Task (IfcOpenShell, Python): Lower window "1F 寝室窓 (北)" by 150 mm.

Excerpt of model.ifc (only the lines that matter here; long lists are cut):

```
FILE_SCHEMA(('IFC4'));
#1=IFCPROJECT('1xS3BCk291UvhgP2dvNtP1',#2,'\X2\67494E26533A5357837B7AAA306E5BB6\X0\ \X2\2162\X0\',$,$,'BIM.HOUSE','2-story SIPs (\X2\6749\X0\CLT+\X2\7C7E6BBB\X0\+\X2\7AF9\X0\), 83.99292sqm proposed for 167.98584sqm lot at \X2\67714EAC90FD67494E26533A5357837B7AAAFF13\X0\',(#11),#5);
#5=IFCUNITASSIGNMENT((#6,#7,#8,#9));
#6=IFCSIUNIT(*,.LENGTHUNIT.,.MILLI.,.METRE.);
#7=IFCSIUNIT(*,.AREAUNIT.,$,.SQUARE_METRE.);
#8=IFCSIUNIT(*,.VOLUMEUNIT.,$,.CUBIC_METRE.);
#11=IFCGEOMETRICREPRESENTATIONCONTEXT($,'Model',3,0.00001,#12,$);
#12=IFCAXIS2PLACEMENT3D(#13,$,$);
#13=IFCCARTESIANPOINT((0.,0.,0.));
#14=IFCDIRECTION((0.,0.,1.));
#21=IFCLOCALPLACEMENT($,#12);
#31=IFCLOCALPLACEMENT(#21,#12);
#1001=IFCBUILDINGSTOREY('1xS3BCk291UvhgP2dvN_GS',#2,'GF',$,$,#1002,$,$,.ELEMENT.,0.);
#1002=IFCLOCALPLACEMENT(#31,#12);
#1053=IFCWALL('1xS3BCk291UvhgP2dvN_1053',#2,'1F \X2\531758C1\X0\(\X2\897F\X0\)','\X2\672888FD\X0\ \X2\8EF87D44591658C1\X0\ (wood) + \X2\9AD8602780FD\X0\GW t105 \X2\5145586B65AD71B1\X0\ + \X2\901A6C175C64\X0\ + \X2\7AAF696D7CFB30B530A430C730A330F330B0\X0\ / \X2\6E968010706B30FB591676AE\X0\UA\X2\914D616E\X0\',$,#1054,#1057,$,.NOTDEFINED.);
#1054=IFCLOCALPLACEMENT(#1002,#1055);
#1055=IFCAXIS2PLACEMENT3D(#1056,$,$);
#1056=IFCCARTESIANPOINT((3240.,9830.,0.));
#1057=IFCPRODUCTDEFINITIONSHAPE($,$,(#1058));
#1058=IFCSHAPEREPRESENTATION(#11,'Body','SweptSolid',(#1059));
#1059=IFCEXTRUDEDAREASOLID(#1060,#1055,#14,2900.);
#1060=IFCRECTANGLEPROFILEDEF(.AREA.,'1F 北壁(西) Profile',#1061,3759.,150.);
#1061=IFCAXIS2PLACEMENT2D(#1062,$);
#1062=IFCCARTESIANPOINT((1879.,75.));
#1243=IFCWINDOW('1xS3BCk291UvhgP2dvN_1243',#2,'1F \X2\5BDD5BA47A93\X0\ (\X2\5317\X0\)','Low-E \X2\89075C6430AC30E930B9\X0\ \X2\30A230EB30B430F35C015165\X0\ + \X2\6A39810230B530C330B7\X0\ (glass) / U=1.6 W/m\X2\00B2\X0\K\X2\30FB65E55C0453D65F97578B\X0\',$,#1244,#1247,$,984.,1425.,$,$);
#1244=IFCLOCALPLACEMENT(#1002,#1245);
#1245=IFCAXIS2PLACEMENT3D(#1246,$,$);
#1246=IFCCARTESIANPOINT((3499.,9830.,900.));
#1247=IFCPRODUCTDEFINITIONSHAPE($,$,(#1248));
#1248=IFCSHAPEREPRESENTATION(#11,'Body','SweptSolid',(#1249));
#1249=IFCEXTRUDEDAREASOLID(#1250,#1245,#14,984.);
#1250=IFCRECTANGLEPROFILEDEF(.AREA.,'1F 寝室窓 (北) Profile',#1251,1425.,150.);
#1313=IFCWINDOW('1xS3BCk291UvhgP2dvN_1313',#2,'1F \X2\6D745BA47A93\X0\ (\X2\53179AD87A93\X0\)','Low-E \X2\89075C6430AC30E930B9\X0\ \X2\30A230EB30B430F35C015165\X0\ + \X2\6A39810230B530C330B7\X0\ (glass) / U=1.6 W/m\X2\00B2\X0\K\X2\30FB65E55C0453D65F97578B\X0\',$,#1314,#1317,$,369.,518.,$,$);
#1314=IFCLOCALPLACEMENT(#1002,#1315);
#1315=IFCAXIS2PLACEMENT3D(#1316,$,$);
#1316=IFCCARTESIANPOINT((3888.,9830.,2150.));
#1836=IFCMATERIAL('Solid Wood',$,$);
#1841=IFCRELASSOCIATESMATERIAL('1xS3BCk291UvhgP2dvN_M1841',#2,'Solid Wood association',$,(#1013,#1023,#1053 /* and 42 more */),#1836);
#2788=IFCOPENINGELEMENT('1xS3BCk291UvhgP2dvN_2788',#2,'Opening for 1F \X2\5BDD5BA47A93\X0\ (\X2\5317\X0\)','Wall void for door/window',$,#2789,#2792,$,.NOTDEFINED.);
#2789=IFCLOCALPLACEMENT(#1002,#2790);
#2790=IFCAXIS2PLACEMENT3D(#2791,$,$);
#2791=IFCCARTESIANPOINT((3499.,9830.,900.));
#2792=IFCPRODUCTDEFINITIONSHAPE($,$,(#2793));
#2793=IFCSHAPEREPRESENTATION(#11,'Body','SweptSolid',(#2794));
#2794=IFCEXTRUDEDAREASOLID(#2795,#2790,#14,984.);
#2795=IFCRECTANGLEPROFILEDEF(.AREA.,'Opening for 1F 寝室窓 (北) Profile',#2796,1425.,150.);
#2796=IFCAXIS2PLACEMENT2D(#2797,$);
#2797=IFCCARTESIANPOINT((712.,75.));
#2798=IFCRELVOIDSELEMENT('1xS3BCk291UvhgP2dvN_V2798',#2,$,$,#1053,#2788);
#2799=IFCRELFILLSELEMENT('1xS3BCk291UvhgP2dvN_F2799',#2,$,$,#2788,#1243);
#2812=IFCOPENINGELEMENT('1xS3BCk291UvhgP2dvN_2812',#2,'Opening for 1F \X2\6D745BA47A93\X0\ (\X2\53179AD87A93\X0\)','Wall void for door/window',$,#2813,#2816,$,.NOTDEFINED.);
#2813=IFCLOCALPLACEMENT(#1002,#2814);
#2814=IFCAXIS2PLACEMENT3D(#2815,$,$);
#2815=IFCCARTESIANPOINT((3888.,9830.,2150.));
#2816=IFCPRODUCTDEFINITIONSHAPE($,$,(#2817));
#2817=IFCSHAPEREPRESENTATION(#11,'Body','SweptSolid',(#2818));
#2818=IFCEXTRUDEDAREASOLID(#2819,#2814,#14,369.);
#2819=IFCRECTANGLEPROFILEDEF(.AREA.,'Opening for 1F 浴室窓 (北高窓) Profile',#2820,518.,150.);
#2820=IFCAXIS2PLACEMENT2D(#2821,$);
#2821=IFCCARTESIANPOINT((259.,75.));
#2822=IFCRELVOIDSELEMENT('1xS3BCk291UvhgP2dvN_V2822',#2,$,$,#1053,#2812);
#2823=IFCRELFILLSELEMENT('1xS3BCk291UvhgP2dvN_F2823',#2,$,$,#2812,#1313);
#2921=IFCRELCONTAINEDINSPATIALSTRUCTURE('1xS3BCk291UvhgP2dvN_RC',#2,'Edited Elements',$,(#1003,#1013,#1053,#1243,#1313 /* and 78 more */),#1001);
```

```python
import numpy as np
import ifcopenshell
import ifcopenshell.api.geometry
import ifcopenshell.util.placement
import ifcopenshell.util.unit

model = ifcopenshell.open("model.ifc")
unit_scale = ifcopenshell.util.unit.calculate_unit_scale(model)

window = model.by_guid("1xS3BCk291UvhgP2dvN_1243")
opening = window.FillsVoids[0].RelatingOpeningElement
dz = -150.0

shift = np.array([0.0, 0.0, dz])
# The window is not placed relative to its opening, so move both.
for product in (opening, window):
    matrix = ifcopenshell.util.placement.get_local_placement(product.ObjectPlacement)
    matrix[:3, 3] += shift
    ifcopenshell.api.geometry.edit_object_placement(model, product=product, matrix=matrix, is_si=False)

print(f"moved by {dz * unit_scale:+.3f} m")

model.write("model_edited.ifc")
```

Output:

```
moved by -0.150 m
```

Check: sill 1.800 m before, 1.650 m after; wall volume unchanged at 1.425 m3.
